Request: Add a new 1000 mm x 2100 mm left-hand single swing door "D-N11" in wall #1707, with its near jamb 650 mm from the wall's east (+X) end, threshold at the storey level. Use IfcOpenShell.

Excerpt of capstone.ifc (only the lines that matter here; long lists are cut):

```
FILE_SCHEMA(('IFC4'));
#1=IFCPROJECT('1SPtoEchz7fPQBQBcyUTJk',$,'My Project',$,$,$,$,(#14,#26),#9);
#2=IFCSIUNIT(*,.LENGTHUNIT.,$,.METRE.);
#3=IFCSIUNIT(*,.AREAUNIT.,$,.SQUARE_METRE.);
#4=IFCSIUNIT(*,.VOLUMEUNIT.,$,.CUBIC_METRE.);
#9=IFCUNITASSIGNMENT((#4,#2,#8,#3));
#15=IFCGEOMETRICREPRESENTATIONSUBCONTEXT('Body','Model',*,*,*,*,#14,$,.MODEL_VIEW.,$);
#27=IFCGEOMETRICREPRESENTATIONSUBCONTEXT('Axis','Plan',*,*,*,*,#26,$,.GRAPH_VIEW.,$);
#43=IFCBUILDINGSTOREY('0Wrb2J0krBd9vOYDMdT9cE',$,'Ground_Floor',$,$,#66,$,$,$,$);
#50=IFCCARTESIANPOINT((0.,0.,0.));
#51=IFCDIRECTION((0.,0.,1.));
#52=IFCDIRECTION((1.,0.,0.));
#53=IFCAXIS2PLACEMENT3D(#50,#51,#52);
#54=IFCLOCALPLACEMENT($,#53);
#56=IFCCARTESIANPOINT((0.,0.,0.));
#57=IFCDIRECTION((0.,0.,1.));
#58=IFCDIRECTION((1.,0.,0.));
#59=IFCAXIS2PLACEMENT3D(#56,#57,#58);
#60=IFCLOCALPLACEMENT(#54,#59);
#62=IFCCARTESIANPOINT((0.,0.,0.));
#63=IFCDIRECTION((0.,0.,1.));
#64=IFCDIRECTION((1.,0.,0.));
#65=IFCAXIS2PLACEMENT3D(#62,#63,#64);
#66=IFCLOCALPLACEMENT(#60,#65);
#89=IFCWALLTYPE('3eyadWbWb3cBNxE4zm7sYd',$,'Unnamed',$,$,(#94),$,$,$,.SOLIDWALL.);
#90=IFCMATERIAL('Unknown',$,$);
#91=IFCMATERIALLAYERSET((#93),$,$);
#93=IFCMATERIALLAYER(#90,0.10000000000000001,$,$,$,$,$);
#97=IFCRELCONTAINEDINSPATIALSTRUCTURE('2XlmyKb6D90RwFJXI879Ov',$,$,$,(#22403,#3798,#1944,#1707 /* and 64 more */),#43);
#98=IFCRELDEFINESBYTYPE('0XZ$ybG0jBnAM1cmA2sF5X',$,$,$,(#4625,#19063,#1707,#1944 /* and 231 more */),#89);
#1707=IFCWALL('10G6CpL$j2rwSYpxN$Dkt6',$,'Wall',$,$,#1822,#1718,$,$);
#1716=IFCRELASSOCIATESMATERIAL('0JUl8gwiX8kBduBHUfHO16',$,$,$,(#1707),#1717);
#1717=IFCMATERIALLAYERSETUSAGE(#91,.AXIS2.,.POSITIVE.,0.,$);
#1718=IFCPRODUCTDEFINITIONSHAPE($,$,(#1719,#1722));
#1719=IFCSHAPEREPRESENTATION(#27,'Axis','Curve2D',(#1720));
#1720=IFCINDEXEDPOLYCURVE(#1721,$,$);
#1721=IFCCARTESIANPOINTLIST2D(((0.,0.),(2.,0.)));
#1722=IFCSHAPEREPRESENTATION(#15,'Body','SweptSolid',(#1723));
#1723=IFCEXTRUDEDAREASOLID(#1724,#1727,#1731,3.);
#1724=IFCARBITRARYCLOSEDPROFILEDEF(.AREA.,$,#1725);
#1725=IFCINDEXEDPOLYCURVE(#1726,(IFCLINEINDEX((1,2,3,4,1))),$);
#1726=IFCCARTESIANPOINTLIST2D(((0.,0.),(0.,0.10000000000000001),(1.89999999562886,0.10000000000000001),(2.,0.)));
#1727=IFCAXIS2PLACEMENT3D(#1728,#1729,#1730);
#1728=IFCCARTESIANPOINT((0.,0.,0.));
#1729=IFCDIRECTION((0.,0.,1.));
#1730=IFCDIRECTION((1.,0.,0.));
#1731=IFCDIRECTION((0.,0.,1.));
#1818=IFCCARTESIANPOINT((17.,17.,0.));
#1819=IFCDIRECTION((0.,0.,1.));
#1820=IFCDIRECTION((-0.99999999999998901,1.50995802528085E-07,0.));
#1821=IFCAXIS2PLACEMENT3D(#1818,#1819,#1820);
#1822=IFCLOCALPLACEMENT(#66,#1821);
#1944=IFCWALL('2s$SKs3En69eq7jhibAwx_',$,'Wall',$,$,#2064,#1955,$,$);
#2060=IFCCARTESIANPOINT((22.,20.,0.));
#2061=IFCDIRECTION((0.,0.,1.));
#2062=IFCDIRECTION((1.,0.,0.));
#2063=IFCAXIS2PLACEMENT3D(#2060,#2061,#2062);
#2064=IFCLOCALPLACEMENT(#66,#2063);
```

```python
import numpy as np
import ifcopenshell
import ifcopenshell.api.feature
import ifcopenshell.api.geometry
import ifcopenshell.api.root
import ifcopenshell.api.spatial
import ifcopenshell.geom
import ifcopenshell.util.element
import ifcopenshell.util.placement
import ifcopenshell.util.representation
import ifcopenshell.util.shape
import ifcopenshell.util.unit

model = ifcopenshell.open("capstone.ifc")
unit_scale = ifcopenshell.util.unit.calculate_unit_scale(model)
settings = ifcopenshell.geom.settings()


def volume(element):
    """Net volume in cubic metres, openings subtracted."""
    shape = ifcopenshell.geom.create_shape(settings, element)
    return ifcopenshell.util.shape.get_volume(shape.geometry)


wall = model.by_id(1707)
storey = ifcopenshell.util.element.get_container(wall, ifc_class="IfcBuildingStorey")
context = ifcopenshell.util.representation.get_context(model, "Model", "Body", "MODEL_VIEW")
before = volume(wall)

width, height, from_end, sill = 1, 2.1, 0.65, 0.0  # metres

# The wall runs along its own X axis, and the end named is its -X end.
wall_shape = ifcopenshell.geom.create_shape(settings, wall)
x, y, z = ifcopenshell.util.shape.get_vertices(wall_shape.geometry).T
start = x.min() + from_end
face, thickness = float(y.min()), float(y.max() - y.min())
wall_matrix = ifcopenshell.util.placement.get_local_placement(wall.ObjectPlacement)
level = ifcopenshell.util.placement.get_local_placement(storey.ObjectPlacement)[2, 3]


def in_wall(x, y):
    """Placement at x, y metres in the wall's axes, at sill height."""
    matrix = wall_matrix.copy()
    matrix[:, 3] = wall_matrix @ np.array([x / unit_scale, y / unit_scale, 0.0, 1.0])
    matrix[2, 3] = level + sill / unit_scale
    return matrix


# Opening: a box that overshoots both wall faces by 50 mm.
opening = ifcopenshell.api.root.create_entity(model, ifc_class="IfcOpeningElement", predefined_type="OPENING")
box = ifcopenshell.api.geometry.add_wall_representation(
    model, context=context, length=width, height=height, thickness=thickness + 0.1
)
ifcopenshell.api.geometry.assign_representation(model, product=opening, representation=box)
ifcopenshell.api.geometry.edit_object_placement(model, product=opening, matrix=in_wall(start, face - 0.05), is_si=False)
ifcopenshell.api.feature.add_feature(model, feature=opening, element=wall)

door = ifcopenshell.api.root.create_entity(model, ifc_class="IfcDoor", name="D-N11", predefined_type="DOOR")
door.OverallWidth, door.OverallHeight = width / unit_scale, height / unit_scale
door.OperationType = "SINGLE_SWING_LEFT"
body = ifcopenshell.api.geometry.add_door_representation(
    model,
    context=context,
    overall_width=door.OverallWidth,
    overall_height=door.OverallHeight,
    operation_type="SINGLE_SWING_LEFT",
    lining_properties={"LiningDepth": thickness / unit_scale, "ThresholdDepth": thickness / unit_scale},
)
ifcopenshell.api.geometry.assign_representation(model, product=door, representation=body)
ifcopenshell.api.spatial.assign_container(model, products=[door], relating_structure=storey)
ifcopenshell.api.feature.add_filling(model, opening=opening, element=door)

# The lining spans the wall, so the door starts at the wall face.
ifcopenshell.api.geometry.edit_object_placement(model, product=door, matrix=in_wall(start, face), is_si=False)

after = volume(wall)

print(f"wall volume {before:.3f} -> {after:.3f} m3")

model.write("capstone_edited.ifc")
```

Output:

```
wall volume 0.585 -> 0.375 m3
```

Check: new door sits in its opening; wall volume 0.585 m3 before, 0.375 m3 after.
